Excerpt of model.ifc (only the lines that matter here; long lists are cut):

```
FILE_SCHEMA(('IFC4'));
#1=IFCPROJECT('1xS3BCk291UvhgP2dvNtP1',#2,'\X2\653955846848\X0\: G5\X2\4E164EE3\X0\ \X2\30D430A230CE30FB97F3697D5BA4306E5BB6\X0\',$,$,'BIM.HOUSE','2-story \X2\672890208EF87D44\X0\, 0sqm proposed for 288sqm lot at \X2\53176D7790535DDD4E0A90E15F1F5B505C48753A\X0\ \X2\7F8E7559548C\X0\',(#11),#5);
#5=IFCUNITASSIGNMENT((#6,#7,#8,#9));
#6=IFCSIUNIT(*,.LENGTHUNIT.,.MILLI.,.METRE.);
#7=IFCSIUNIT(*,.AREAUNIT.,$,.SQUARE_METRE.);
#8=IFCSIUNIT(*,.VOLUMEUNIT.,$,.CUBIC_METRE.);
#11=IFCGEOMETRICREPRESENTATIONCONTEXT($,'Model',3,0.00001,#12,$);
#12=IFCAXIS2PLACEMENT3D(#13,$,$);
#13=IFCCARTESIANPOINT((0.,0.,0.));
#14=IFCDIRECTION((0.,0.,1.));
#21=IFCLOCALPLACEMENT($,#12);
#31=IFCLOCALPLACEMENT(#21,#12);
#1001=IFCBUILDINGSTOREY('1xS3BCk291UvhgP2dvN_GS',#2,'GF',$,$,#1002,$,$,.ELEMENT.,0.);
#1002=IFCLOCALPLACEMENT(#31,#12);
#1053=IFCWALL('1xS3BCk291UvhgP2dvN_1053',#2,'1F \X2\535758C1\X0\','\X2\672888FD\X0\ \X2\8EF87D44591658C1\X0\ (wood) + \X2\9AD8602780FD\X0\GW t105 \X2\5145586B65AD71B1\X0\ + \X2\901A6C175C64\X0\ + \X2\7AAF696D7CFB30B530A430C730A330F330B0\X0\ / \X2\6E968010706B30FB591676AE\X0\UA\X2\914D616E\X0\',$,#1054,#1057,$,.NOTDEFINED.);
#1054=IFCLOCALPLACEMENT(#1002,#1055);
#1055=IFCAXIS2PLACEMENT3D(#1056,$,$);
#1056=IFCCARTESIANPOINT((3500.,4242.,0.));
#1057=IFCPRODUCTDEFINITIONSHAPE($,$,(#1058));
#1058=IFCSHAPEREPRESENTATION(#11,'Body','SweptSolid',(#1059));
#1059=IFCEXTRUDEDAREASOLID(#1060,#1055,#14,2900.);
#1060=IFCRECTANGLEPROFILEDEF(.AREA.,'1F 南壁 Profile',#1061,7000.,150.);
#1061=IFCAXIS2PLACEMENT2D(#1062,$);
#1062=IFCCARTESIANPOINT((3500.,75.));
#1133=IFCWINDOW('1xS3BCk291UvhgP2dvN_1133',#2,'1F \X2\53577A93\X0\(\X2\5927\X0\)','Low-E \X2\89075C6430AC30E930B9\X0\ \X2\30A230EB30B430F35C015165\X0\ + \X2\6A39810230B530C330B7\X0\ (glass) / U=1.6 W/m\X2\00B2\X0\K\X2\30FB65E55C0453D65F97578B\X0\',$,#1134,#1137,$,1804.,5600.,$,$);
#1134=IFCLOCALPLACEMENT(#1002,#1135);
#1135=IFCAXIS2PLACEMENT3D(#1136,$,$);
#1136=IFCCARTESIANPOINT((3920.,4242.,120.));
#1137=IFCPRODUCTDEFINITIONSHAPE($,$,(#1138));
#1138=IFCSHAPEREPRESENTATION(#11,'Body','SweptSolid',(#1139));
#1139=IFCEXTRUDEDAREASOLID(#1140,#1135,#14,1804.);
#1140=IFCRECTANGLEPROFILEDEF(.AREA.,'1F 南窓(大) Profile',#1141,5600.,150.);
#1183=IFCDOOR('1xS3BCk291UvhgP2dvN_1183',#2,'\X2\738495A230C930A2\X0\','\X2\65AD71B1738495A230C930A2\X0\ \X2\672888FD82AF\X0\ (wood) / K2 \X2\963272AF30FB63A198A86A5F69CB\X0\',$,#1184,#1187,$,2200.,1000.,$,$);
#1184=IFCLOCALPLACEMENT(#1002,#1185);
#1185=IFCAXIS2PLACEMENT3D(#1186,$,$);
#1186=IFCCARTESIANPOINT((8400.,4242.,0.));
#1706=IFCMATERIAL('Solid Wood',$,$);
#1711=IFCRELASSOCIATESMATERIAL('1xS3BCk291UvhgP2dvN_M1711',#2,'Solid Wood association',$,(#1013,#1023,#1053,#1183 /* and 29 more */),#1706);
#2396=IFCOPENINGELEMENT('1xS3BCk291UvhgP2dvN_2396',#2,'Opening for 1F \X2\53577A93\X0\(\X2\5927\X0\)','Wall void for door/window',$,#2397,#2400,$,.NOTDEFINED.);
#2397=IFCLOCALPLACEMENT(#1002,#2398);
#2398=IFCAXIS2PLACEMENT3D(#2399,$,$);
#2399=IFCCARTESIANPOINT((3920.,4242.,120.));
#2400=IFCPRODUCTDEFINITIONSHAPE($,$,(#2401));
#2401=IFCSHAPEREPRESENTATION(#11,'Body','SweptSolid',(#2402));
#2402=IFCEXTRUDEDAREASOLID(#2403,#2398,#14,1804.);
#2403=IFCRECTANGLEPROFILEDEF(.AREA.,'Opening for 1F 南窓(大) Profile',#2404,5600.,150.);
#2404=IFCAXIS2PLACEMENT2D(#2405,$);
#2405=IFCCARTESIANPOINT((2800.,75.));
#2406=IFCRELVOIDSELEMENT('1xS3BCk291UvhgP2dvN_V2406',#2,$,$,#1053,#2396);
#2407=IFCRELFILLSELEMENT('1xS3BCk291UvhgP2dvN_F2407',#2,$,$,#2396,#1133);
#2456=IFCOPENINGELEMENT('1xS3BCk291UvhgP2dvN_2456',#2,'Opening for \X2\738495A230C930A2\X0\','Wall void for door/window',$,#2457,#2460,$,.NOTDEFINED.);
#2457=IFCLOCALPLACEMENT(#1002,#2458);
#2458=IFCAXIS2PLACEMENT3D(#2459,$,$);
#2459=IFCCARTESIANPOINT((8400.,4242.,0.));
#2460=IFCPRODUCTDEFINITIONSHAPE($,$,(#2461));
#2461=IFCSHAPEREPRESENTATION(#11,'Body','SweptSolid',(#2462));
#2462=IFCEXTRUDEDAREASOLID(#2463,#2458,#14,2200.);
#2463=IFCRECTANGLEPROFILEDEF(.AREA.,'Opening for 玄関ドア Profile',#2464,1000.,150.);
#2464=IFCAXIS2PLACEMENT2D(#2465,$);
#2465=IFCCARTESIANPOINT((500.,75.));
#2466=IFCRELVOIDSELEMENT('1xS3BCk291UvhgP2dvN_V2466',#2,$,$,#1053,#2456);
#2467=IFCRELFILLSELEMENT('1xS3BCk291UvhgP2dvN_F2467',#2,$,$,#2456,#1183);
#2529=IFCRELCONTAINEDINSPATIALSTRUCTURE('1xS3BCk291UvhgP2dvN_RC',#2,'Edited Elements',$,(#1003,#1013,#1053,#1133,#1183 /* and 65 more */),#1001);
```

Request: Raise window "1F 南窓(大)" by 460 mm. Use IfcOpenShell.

```python
import numpy as np
import ifcopenshell
import ifcopenshell.api.geometry
import ifcopenshell.util.placement
import ifcopenshell.util.unit

model = ifcopenshell.open("model.ifc")
unit_scale = ifcopenshell.util.unit.calculate_unit_scale(model)

window = model.by_id(1133)
opening = window.FillsVoids[0].RelatingOpeningElement
dz = 460.0

shift = np.array([0.0, 0.0, dz])
# The window is not placed relative to its opening, so move both.
for product in (opening, window):
    matrix = ifcopenshell.util.placement.get_local_placement(product.ObjectPlacement)
    matrix[:3, 3] += shift
    ifcopenshell.api.geometry.edit_object_placement(model, product=product, matrix=matrix, is_si=False)

print(f"moved by {dz * unit_scale:+.3f} m")

model.write("model_v2.ifc")
```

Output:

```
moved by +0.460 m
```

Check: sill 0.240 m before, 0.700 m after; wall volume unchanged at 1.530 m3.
